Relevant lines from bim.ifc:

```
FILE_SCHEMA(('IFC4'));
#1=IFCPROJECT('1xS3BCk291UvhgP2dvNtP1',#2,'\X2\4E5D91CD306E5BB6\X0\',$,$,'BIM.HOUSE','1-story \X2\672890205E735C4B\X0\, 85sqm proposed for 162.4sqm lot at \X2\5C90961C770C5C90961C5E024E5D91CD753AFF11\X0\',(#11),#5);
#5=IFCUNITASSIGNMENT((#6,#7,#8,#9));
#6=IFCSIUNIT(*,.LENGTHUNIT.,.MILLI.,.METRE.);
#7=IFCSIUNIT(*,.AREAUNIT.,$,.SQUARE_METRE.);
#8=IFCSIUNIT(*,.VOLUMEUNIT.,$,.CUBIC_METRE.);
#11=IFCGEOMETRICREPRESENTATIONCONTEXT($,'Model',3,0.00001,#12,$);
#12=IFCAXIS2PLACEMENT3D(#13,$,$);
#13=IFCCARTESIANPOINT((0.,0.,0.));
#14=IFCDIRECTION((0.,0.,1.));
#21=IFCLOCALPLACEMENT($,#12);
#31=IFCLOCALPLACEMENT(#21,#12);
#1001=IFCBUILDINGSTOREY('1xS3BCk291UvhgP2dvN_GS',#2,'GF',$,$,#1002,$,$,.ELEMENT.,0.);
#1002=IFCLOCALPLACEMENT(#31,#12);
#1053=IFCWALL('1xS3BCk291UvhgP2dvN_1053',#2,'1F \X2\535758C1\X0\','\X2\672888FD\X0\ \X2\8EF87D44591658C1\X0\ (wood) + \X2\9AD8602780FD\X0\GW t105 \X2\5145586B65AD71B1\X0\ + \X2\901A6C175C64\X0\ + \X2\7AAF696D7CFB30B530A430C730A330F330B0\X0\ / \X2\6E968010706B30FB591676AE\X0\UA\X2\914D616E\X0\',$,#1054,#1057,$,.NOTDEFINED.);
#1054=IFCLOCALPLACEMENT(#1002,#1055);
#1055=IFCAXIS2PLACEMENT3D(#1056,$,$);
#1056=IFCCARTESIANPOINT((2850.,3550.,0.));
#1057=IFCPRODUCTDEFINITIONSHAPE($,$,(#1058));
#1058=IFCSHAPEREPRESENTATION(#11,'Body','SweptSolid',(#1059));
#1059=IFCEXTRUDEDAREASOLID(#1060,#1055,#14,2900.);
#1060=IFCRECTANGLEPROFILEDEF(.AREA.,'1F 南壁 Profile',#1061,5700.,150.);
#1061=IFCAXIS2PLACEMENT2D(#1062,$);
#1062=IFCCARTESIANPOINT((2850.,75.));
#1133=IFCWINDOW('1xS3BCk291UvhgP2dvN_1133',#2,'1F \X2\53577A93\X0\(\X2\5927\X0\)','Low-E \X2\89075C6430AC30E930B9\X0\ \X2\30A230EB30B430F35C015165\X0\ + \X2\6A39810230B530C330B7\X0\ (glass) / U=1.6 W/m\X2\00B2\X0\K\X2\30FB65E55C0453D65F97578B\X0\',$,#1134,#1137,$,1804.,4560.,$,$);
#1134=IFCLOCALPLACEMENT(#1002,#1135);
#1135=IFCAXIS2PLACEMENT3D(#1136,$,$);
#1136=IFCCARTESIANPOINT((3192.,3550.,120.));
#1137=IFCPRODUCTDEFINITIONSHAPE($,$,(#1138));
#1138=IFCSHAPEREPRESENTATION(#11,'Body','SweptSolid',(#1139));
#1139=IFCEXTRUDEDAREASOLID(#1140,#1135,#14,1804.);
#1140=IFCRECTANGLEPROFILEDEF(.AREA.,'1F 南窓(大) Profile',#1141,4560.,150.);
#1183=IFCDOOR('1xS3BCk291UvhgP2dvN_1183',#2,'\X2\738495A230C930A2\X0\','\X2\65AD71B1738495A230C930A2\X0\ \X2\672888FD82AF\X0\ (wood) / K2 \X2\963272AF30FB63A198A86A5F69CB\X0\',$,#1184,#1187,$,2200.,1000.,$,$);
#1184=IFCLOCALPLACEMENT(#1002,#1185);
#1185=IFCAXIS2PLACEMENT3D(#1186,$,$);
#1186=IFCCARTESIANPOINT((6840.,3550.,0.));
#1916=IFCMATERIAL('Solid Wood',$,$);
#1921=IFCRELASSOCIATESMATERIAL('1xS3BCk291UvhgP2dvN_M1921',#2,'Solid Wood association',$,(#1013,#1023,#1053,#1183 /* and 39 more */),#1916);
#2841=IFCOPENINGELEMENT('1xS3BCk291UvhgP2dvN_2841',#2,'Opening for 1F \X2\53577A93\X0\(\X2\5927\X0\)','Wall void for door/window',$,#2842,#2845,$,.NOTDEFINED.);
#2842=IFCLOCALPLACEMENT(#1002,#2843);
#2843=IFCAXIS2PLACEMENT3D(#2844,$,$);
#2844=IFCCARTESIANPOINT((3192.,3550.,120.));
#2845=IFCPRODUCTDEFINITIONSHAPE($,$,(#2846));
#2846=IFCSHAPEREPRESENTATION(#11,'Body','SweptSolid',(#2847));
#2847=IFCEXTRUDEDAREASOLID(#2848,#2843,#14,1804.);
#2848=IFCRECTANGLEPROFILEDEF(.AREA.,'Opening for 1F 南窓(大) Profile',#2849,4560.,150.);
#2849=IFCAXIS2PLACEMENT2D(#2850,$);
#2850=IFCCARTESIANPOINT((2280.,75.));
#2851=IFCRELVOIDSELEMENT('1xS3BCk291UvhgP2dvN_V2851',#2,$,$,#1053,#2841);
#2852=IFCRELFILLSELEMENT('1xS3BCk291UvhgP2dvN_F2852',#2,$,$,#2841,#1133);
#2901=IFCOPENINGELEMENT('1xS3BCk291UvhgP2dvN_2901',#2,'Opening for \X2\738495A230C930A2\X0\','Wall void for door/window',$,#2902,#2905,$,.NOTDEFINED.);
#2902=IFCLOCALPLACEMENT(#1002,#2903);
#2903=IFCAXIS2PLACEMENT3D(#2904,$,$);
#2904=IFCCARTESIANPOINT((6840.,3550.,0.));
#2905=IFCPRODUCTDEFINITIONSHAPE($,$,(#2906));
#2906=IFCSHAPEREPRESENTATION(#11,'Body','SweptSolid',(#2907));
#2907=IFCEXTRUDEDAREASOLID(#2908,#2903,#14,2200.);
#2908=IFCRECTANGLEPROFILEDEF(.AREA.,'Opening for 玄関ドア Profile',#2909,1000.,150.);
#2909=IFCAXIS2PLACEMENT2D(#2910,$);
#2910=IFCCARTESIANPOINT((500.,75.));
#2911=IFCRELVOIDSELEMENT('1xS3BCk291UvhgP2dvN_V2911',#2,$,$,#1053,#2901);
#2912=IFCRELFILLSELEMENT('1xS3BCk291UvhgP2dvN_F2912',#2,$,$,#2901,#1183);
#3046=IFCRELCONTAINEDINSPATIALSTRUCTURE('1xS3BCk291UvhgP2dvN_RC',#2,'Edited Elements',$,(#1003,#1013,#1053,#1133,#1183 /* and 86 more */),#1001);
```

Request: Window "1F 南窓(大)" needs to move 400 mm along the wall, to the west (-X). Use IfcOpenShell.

```python
import ifcopenshell
import ifcopenshell.api.geometry
import ifcopenshell.util.placement

model = ifcopenshell.open("bim.ifc")

window = model.by_id(1133)
opening = window.FillsVoids[0].RelatingOpeningElement
wall = opening.VoidsElements[0].RelatingBuildingElement

wall_matrix = ifcopenshell.util.placement.get_local_placement(wall.ObjectPlacement)
shift = wall_matrix[:3, 0] * -400.0
before = ifcopenshell.util.placement.get_local_placement(window.ObjectPlacement)[:3, 3].copy()

# The window is not placed relative to its opening, so move both.
for product in (opening, window):
    matrix = ifcopenshell.util.placement.get_local_placement(product.ObjectPlacement)
    matrix[:3, 3] += shift
    ifcopenshell.api.geometry.edit_object_placement(model, product=product, matrix=matrix, is_si=False)

after = ifcopenshell.util.placement.get_local_placement(window.ObjectPlacement)[:3, 3]
print("window moved by", (after - before).round(3) + 0.0)

model.write("bim_v2.ifc")
```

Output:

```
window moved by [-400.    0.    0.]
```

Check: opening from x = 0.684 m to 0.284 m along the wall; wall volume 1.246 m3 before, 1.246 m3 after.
